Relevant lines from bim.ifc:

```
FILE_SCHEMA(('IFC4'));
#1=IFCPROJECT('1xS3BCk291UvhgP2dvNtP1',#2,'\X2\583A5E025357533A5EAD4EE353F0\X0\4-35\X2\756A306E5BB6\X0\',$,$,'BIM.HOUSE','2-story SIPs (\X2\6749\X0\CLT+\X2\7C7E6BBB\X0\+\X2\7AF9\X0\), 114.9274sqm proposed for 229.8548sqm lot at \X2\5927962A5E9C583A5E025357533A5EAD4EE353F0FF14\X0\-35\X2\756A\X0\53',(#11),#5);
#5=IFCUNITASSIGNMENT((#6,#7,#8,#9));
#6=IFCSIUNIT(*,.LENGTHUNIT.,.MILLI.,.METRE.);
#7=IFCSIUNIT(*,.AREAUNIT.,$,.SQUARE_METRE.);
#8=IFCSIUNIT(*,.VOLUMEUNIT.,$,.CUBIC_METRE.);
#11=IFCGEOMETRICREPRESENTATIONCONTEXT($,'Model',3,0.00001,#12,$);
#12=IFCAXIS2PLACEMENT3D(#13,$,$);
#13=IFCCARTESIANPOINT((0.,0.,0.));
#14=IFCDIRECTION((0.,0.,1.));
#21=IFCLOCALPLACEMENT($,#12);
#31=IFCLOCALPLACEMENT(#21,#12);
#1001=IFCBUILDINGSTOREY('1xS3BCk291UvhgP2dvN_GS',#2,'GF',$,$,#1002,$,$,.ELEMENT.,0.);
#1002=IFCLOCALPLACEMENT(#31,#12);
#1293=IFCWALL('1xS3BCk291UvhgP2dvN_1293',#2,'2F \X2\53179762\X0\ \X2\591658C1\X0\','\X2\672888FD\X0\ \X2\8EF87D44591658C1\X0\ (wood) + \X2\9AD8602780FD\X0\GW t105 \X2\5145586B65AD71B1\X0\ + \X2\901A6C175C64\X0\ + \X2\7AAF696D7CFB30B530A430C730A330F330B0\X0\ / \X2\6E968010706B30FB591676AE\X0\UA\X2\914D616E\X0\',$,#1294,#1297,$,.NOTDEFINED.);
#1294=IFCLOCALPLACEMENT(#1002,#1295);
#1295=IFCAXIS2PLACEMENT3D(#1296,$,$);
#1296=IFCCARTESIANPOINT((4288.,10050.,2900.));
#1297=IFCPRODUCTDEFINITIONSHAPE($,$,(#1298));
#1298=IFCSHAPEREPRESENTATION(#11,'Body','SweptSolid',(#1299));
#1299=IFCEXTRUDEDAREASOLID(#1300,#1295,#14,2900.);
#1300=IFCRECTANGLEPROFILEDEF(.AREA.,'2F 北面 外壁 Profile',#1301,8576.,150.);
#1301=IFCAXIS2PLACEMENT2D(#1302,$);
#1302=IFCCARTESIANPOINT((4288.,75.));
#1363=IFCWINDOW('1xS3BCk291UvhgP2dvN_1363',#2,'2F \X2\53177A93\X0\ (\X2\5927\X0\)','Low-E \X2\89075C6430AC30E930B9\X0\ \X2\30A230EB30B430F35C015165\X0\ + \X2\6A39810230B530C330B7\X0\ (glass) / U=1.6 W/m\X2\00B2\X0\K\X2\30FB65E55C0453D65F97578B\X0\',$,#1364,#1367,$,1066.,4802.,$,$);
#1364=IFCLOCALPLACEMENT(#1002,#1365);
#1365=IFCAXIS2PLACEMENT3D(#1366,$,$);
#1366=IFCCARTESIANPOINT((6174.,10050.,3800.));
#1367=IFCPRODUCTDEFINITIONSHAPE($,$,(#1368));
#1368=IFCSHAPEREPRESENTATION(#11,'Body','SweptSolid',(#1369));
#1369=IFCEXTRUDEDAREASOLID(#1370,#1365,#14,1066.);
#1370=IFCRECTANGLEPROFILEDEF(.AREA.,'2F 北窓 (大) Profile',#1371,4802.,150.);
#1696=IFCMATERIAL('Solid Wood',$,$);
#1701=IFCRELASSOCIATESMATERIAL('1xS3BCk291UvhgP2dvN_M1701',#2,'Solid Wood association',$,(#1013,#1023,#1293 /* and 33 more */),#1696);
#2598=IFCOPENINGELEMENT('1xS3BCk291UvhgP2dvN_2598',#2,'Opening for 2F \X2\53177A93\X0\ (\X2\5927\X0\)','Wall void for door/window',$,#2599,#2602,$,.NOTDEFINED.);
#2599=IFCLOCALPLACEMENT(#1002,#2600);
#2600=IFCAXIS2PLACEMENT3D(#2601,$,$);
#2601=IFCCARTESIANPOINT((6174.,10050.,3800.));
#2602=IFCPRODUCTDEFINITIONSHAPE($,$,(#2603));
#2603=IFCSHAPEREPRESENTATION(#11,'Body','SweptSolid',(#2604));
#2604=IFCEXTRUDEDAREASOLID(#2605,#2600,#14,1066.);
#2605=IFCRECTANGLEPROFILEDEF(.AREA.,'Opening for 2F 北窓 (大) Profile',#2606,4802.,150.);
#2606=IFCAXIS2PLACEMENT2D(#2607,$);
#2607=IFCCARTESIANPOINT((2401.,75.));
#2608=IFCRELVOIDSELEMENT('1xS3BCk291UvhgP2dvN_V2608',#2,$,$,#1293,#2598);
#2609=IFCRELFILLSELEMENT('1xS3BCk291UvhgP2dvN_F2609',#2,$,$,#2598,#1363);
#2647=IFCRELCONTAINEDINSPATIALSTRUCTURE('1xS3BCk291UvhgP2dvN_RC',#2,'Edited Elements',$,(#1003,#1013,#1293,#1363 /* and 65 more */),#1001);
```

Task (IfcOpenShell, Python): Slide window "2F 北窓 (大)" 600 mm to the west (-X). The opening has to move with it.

```python
import ifcopenshell
import ifcopenshell.api.geometry
import ifcopenshell.util.placement

model = ifcopenshell.open("bim.ifc")

window = model.by_id(1363)
opening = window.FillsVoids[0].RelatingOpeningElement
wall = opening.VoidsElements[0].RelatingBuildingElement

wall_matrix = ifcopenshell.util.placement.get_local_placement(wall.ObjectPlacement)
shift = wall_matrix[:3, 0] * -600.0
before = ifcopenshell.util.placement.get_local_placement(window.ObjectPlacement)[:3, 3].copy()

# The window is not placed relative to its opening, so move both.
for product in (opening, window):
    matrix = ifcopenshell.util.placement.get_local_placement(product.ObjectPlacement)
    matrix[:3, 3] += shift
    ifcopenshell.api.geometry.edit_object_placement(model, product=product, matrix=matrix, is_si=False)

after = ifcopenshell.util.placement.get_local_placement(window.ObjectPlacement)[:3, 3]
print("window moved by", (after - before).round(3) + 0.0)

model.write("bim_v2.ifc")
```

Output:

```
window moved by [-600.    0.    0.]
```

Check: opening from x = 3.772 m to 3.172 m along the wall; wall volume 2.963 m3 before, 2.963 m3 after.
